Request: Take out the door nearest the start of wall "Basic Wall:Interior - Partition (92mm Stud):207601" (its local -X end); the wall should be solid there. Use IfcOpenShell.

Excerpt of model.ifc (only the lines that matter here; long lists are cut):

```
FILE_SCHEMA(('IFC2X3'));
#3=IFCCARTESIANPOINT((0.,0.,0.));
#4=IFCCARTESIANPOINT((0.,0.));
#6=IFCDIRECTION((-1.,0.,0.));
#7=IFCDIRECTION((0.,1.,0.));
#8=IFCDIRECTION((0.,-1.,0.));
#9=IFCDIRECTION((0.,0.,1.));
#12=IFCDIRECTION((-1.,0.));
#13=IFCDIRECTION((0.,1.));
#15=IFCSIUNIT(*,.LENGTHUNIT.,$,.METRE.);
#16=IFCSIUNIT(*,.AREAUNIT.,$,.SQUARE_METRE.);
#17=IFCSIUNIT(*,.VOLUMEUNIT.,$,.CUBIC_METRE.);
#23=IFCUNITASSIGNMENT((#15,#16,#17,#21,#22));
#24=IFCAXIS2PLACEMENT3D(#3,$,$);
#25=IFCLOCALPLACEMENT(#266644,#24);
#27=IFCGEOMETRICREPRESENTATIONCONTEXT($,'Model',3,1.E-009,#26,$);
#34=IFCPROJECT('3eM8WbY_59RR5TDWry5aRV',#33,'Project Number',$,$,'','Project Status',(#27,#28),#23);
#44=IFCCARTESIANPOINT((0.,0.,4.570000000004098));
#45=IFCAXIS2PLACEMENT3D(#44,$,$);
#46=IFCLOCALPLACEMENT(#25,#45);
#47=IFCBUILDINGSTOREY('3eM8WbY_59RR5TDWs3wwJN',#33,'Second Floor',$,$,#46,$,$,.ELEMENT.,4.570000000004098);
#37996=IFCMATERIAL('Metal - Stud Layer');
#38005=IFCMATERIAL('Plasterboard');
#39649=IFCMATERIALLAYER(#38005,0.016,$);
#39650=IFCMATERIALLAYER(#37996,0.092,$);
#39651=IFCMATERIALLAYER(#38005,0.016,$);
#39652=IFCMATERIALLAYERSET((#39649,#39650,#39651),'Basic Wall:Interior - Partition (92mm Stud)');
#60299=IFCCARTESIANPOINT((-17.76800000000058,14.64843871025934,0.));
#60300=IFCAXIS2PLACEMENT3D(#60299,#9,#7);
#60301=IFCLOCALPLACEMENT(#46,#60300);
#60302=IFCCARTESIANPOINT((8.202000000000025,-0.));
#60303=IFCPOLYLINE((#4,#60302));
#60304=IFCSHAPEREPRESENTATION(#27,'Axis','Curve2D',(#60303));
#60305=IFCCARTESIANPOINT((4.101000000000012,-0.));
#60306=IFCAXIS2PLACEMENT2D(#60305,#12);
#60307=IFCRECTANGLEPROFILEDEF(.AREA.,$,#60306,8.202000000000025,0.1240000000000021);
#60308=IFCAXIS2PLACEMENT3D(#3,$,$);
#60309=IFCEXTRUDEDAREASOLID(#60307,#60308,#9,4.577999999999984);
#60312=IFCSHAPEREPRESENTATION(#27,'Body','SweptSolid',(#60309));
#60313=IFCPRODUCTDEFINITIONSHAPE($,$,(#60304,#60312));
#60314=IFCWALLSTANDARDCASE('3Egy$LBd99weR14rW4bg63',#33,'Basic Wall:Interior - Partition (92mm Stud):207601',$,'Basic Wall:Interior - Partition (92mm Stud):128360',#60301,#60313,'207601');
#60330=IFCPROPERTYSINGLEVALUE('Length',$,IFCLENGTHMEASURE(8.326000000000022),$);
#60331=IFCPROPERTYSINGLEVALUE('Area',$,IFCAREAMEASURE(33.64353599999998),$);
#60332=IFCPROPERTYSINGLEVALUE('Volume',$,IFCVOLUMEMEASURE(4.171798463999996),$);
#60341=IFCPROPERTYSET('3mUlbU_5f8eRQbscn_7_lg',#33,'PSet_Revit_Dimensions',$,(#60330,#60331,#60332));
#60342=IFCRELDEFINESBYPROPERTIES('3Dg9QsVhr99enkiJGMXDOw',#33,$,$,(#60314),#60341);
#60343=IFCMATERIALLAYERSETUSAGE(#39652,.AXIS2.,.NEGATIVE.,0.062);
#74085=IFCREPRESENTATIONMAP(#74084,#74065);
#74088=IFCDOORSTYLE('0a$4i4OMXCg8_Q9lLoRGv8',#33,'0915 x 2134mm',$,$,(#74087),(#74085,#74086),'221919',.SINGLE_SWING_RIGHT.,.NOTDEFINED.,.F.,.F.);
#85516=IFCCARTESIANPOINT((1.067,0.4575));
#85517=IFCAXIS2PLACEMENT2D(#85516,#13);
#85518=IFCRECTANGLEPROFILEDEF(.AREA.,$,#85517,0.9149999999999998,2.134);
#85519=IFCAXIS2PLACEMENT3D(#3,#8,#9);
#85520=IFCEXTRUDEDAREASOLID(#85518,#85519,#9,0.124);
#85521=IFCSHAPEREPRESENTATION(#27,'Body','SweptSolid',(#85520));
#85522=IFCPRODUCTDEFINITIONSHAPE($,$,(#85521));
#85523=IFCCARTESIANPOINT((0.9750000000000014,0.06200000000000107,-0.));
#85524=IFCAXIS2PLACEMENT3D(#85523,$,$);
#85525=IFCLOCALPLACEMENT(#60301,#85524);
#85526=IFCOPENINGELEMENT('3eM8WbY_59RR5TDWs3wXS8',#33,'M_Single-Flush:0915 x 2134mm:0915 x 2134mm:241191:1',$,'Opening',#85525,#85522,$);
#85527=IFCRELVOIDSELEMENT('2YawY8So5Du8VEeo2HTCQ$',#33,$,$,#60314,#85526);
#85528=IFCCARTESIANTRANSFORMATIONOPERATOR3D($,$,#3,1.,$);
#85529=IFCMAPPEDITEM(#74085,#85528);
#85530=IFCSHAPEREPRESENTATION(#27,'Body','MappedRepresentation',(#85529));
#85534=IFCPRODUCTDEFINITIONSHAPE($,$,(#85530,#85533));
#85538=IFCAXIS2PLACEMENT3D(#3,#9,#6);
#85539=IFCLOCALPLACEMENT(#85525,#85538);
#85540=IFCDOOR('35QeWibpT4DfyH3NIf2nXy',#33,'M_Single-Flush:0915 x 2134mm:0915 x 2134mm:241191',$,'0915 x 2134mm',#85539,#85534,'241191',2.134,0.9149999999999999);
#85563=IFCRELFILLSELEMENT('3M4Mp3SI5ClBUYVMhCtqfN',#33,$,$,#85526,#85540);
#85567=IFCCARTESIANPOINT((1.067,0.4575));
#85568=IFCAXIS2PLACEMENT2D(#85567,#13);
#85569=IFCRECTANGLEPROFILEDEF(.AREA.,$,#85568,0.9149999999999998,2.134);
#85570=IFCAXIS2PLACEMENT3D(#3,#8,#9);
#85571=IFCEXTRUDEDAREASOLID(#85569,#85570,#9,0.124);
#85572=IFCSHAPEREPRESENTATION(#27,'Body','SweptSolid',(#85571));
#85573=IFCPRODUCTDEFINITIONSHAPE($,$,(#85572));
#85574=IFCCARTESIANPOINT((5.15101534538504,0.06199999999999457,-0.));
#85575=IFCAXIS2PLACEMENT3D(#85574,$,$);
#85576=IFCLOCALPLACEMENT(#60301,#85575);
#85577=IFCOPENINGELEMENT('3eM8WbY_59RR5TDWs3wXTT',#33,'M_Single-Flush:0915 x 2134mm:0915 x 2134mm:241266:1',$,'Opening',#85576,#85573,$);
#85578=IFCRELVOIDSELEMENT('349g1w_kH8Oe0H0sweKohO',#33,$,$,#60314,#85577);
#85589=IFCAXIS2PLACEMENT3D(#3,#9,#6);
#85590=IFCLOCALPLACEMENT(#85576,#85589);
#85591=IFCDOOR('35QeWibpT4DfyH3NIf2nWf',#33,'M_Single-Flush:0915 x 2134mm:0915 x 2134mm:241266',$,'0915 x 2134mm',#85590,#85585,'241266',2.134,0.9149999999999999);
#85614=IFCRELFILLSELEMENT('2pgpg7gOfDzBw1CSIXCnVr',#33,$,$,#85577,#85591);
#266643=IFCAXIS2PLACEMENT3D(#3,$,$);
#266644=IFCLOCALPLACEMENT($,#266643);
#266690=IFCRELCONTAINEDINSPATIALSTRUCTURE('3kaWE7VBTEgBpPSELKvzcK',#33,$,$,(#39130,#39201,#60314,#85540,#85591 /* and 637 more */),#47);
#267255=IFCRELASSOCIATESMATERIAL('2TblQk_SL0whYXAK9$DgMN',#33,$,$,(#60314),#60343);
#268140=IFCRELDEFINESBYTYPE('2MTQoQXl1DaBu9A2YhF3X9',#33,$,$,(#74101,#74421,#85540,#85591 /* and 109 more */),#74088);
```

```python
import ifcopenshell
import ifcopenshell.api.feature
import ifcopenshell.api.pset
import ifcopenshell.api.root
import ifcopenshell.geom
import ifcopenshell.util.element
import ifcopenshell.util.shape
import ifcopenshell.util.unit

model = ifcopenshell.open("model.ifc")
area_scale = ifcopenshell.util.unit.calculate_unit_scale(model, "AREAUNIT")
volume_scale = ifcopenshell.util.unit.calculate_unit_scale(model, "VOLUMEUNIT")
settings = ifcopenshell.geom.settings()


def volume(element):
    """Net volume in cubic metres, openings subtracted."""
    shape = ifcopenshell.geom.create_shape(settings, element)
    return ifcopenshell.util.shape.get_volume(shape.geometry)


door = model.by_id(85540)
opening = door.FillsVoids[0].RelatingOpeningElement
wall = opening.VoidsElements[0].RelatingBuildingElement
before = volume(wall)

ifcopenshell.api.root.remove_product(model, product=door)
ifcopenshell.api.feature.remove_feature(model, feature=opening)

after = volume(wall)
thickness = 0.124  # wall thickness in metres

# Update the wall's stored quantities.
pset = model.by_id(ifcopenshell.util.element.get_pset(wall, "PSet_Revit_Dimensions", should_inherit=False)["id"])
ifcopenshell.api.pset.edit_pset(model, pset=pset, properties={
    "Area": model.create_entity("IfcAreaMeasure", after / thickness / area_scale),
    "Volume": model.create_entity("IfcVolumeMeasure", after / volume_scale),
})

print(f"wall volume {before:.3f} -> {after:.3f} m3")

model.write("model_v2.ifc")
```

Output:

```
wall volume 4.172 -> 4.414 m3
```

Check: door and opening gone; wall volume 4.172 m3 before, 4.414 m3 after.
